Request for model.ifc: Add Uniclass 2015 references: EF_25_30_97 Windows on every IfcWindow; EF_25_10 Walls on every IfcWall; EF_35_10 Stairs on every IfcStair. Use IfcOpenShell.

First a look at what the model holds.

```python
import ifcopenshell

model = ifcopenshell.open("model.ifc")
print(model.schema)
print("classifications:", [c.Name for c in model.by_type("IfcClassification")])
for ifc_class in ("IfcDoor", "IfcRoof", "IfcStair", "IfcWall", "IfcWindow"):
    print(ifc_class, len(model.by_type(ifc_class)))
```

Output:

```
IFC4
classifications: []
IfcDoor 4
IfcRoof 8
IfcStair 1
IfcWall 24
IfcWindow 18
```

```python
import ifcopenshell
import ifcopenshell.api.classification

model = ifcopenshell.open("model.ifc")

system = ifcopenshell.api.classification.add_classification(model, classification="Uniclass 2015")

codes = {
    "IfcWindow": ("EF_25_30_97", "Windows"),
    "IfcWall": ("EF_25_10", "Walls"),
    "IfcStair": ("EF_35_10", "Stairs"),
}
for ifc_class, (code, name) in codes.items():
    products = model.by_type(ifc_class)
    ifcopenshell.api.classification.add_reference(
        model, products=products, classification=system, identification=code, name=name
    )
    print(code, len(products))

model.write("model_rev.ifc")
```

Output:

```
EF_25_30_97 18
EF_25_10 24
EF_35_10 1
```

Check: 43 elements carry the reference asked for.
